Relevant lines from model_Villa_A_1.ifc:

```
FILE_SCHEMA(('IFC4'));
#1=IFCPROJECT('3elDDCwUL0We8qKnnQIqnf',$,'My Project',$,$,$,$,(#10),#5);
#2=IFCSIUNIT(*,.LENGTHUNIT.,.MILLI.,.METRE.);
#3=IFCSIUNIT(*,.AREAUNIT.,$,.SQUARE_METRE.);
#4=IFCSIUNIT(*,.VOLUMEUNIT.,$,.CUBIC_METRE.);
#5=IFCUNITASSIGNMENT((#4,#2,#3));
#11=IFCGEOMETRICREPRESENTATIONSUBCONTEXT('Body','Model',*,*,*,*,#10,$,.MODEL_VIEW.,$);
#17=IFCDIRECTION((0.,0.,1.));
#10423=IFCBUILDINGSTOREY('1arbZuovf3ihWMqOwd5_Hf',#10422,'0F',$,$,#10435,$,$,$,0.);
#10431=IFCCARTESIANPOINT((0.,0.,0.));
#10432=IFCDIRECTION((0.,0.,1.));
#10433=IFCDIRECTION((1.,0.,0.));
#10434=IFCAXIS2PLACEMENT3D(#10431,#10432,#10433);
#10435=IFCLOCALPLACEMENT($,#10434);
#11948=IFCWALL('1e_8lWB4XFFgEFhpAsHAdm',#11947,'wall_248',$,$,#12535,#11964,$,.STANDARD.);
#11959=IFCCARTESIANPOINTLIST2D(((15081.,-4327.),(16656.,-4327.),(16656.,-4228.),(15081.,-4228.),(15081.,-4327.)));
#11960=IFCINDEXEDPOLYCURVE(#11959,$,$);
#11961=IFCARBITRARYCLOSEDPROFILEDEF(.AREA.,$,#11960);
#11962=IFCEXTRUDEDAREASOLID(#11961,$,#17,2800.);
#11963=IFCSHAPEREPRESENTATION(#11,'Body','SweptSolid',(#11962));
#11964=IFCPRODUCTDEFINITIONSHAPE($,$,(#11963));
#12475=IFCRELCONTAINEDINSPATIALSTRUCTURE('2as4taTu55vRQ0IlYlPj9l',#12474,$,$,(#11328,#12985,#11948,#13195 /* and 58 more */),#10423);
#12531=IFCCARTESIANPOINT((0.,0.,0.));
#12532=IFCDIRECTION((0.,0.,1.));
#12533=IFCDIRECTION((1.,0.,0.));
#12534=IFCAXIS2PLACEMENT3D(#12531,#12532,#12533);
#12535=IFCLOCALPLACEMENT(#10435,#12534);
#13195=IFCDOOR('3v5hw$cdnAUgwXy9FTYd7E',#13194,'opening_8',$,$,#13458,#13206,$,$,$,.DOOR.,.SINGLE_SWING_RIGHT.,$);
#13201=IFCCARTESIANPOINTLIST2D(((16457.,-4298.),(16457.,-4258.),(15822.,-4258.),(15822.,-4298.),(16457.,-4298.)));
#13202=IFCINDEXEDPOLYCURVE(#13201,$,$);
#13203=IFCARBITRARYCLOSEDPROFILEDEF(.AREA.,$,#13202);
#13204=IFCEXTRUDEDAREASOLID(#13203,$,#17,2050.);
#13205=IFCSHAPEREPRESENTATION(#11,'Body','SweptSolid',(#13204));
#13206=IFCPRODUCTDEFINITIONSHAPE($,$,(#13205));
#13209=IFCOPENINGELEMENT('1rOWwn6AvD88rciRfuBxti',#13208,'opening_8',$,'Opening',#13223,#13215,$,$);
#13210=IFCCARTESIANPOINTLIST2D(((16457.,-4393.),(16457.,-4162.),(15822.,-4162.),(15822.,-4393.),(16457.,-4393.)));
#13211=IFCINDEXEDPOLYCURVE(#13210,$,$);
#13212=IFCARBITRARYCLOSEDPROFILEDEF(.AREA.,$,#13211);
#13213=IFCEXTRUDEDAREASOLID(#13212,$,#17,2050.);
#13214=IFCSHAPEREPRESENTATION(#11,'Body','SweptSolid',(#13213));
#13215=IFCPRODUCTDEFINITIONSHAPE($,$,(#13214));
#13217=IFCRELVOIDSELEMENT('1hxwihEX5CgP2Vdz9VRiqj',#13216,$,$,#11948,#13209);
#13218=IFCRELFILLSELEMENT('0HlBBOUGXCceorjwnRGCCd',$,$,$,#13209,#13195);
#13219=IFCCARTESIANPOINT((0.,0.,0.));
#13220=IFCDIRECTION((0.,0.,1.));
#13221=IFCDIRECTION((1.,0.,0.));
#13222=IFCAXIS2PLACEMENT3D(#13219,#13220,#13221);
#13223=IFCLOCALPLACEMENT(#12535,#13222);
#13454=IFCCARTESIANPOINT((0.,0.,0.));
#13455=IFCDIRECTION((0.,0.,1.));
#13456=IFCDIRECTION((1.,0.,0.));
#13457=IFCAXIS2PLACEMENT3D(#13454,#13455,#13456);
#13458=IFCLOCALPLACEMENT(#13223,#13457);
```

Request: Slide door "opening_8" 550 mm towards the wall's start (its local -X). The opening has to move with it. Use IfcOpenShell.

```python
import ifcopenshell
import ifcopenshell.api.geometry
import ifcopenshell.util.placement

model = ifcopenshell.open("model_Villa_A_1.ifc")

door = model.by_guid("3v5hw$cdnAUgwXy9FTYd7E")
opening = door.FillsVoids[0].RelatingOpeningElement
wall = opening.VoidsElements[0].RelatingBuildingElement

wall_matrix = ifcopenshell.util.placement.get_local_placement(wall.ObjectPlacement)
shift = wall_matrix[:3, 0] * -550.0
before = ifcopenshell.util.placement.get_local_placement(door.ObjectPlacement)[:3, 3].copy()

# The door is placed relative to its opening, so it follows when the opening moves.
matrix = ifcopenshell.util.placement.get_local_placement(opening.ObjectPlacement)
matrix[:3, 3] += shift
ifcopenshell.api.geometry.edit_object_placement(
    model, product=opening, matrix=matrix, is_si=False, should_transform_children=True
)

after = ifcopenshell.util.placement.get_local_placement(door.ObjectPlacement)[:3, 3]
print("door moved by", (after - before).round(3) + 0.0)

model.write("model_Villa_A_1_v2.ifc")
```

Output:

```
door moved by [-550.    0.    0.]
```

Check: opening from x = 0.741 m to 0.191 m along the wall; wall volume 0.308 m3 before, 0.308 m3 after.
